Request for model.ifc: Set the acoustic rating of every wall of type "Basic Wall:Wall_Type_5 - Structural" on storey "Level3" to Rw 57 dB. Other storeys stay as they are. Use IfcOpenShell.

First a look at what the model holds.

```python
import ifcopenshell
import ifcopenshell.util.element

model = ifcopenshell.open("model.ifc")
print(model.schema)
storey = next(s for s in model.by_type("IfcBuildingStorey") if s.Name == "Level3")
walls = [e for e in ifcopenshell.util.element.get_decomposition(storey) if e.is_a("IfcWall")]
seen = {}
for e in walls:
    element_type = ifcopenshell.util.element.get_type(e)
    key = (element_type.Name if element_type != e and element_type else None, ifcopenshell.util.element.get_pset(e, "Pset_WallCommon", "AcousticRating"))
    seen[key] = seen.get(key, 0) + 1
for (name, value), count in sorted(seen.items(), key=str):
    print(count, "x", name, "|", value)
```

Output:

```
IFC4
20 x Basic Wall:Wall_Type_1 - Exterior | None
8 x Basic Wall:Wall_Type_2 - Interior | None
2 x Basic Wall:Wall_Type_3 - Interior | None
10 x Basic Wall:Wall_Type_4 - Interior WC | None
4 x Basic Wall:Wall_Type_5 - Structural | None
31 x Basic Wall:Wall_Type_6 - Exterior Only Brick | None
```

```python
import ifcopenshell
import ifcopenshell.api.pset
import ifcopenshell.util.element

model = ifcopenshell.open("model.ifc")

storey = next(s for s in model.by_type("IfcBuildingStorey") if s.Name == "Level3")
walls = [e for e in ifcopenshell.util.element.get_decomposition(storey) if e.is_a("IfcWall")]

count = 0
for e in walls:
    element_type = ifcopenshell.util.element.get_type(e)
    if element_type in (None, e) or element_type.Name != "Basic Wall:Wall_Type_5 - Structural":
        continue
    # add_pset returns the element's existing set when there is one.
    pset = ifcopenshell.api.pset.add_pset(model, product=e, name="Pset_WallCommon")
    ifcopenshell.api.pset.edit_pset(model, pset=pset, properties={"AcousticRating": "Rw 57 dB"})
    count += 1

print(count, "walls updated")

model.write("model-out.ifc")
```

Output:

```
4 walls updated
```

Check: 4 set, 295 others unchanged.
